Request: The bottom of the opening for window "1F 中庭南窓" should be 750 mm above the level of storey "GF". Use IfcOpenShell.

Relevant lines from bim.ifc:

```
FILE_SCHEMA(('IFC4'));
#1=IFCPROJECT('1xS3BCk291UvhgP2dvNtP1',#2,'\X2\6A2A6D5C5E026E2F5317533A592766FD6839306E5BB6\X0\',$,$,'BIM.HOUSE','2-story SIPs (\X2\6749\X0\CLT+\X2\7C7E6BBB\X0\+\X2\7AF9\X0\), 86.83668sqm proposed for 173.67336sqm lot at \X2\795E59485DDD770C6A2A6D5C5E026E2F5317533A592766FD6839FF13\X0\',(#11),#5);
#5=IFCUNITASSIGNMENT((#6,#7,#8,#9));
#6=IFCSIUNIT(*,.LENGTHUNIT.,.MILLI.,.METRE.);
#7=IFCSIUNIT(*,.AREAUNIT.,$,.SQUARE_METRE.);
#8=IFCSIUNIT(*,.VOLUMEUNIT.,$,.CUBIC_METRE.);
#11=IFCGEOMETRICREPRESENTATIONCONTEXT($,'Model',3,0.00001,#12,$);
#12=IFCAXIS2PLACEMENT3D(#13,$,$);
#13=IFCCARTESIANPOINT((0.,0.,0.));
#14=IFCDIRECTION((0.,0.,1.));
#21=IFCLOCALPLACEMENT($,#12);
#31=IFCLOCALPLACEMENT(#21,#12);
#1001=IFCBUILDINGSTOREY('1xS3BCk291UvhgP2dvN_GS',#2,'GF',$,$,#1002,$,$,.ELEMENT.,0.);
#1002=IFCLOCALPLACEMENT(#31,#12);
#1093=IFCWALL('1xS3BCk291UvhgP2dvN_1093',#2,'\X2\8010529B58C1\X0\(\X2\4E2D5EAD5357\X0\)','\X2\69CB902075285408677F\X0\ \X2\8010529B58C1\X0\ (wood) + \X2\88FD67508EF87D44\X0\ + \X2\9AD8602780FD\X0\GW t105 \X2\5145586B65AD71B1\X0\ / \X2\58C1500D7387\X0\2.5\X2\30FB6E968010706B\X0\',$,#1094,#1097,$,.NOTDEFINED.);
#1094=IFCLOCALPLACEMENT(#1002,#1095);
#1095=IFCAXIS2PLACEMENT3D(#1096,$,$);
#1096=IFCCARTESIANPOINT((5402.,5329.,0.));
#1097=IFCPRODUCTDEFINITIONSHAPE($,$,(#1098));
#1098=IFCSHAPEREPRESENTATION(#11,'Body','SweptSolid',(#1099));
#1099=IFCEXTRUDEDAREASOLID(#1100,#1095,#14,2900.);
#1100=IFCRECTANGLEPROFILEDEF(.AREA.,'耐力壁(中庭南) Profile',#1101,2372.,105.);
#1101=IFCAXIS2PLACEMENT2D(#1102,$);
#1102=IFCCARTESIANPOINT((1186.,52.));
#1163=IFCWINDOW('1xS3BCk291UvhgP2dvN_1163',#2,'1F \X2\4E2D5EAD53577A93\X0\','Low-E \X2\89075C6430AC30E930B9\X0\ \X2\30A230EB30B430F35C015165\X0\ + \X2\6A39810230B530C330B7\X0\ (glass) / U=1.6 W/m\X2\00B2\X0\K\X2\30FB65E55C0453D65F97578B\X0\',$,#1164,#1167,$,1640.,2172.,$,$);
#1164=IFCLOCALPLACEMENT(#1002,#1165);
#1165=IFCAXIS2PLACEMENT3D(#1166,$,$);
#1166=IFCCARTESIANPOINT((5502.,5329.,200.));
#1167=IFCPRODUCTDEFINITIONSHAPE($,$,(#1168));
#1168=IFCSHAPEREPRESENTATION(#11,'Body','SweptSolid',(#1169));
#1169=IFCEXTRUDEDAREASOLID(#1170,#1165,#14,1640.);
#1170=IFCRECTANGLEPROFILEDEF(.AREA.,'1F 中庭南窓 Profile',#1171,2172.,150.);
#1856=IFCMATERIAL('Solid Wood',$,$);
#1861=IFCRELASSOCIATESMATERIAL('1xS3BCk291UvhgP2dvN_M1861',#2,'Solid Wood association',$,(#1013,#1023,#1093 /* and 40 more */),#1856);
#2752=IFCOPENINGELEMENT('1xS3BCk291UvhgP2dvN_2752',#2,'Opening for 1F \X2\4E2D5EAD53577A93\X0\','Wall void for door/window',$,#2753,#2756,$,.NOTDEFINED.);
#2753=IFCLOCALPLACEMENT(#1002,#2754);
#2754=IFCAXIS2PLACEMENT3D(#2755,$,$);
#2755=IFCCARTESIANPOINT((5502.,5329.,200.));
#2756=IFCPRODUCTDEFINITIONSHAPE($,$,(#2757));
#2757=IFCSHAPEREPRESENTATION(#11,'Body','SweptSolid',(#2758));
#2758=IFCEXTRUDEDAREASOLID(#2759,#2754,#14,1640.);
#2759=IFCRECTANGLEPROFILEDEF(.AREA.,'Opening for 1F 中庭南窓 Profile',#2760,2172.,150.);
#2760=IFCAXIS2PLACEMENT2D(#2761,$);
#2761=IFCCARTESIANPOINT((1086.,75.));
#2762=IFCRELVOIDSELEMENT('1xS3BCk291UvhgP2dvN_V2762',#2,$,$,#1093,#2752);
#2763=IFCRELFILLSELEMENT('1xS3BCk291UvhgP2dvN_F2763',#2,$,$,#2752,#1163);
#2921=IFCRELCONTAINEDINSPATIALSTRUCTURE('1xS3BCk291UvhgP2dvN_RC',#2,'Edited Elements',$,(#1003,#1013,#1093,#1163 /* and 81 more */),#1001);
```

```python
import numpy as np
import ifcopenshell
import ifcopenshell.api.geometry
import ifcopenshell.geom
import ifcopenshell.util.element
import ifcopenshell.util.placement
import ifcopenshell.util.shape
import ifcopenshell.util.unit

model = ifcopenshell.open("bim.ifc")
unit_scale = ifcopenshell.util.unit.calculate_unit_scale(model)

window = model.by_id(1163)
opening = window.FillsVoids[0].RelatingOpeningElement
storey = ifcopenshell.util.element.get_container(window, ifc_class="IfcBuildingStorey")
level = ifcopenshell.util.placement.get_local_placement(storey.ObjectPlacement)[2, 3]

# The opening's origin need not be at the sill, so measure its lowest point.
shape = ifcopenshell.geom.create_shape(ifcopenshell.geom.settings(), opening)
bottom = ifcopenshell.util.shape.get_shape_bottom_elevation(shape, shape.geometry) / unit_scale
dz = level + 0.75 / unit_scale - bottom

shift = np.array([0.0, 0.0, dz])
# The window is not placed relative to its opening, so move both.
for product in (opening, window):
    matrix = ifcopenshell.util.placement.get_local_placement(product.ObjectPlacement)
    matrix[:3, 3] += shift
    ifcopenshell.api.geometry.edit_object_placement(model, product=product, matrix=matrix, is_si=False)

print(f"moved by {dz * unit_scale:+.3f} m")

model.write("bim_edited.ifc")
```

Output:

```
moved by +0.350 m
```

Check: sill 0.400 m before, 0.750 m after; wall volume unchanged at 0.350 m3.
